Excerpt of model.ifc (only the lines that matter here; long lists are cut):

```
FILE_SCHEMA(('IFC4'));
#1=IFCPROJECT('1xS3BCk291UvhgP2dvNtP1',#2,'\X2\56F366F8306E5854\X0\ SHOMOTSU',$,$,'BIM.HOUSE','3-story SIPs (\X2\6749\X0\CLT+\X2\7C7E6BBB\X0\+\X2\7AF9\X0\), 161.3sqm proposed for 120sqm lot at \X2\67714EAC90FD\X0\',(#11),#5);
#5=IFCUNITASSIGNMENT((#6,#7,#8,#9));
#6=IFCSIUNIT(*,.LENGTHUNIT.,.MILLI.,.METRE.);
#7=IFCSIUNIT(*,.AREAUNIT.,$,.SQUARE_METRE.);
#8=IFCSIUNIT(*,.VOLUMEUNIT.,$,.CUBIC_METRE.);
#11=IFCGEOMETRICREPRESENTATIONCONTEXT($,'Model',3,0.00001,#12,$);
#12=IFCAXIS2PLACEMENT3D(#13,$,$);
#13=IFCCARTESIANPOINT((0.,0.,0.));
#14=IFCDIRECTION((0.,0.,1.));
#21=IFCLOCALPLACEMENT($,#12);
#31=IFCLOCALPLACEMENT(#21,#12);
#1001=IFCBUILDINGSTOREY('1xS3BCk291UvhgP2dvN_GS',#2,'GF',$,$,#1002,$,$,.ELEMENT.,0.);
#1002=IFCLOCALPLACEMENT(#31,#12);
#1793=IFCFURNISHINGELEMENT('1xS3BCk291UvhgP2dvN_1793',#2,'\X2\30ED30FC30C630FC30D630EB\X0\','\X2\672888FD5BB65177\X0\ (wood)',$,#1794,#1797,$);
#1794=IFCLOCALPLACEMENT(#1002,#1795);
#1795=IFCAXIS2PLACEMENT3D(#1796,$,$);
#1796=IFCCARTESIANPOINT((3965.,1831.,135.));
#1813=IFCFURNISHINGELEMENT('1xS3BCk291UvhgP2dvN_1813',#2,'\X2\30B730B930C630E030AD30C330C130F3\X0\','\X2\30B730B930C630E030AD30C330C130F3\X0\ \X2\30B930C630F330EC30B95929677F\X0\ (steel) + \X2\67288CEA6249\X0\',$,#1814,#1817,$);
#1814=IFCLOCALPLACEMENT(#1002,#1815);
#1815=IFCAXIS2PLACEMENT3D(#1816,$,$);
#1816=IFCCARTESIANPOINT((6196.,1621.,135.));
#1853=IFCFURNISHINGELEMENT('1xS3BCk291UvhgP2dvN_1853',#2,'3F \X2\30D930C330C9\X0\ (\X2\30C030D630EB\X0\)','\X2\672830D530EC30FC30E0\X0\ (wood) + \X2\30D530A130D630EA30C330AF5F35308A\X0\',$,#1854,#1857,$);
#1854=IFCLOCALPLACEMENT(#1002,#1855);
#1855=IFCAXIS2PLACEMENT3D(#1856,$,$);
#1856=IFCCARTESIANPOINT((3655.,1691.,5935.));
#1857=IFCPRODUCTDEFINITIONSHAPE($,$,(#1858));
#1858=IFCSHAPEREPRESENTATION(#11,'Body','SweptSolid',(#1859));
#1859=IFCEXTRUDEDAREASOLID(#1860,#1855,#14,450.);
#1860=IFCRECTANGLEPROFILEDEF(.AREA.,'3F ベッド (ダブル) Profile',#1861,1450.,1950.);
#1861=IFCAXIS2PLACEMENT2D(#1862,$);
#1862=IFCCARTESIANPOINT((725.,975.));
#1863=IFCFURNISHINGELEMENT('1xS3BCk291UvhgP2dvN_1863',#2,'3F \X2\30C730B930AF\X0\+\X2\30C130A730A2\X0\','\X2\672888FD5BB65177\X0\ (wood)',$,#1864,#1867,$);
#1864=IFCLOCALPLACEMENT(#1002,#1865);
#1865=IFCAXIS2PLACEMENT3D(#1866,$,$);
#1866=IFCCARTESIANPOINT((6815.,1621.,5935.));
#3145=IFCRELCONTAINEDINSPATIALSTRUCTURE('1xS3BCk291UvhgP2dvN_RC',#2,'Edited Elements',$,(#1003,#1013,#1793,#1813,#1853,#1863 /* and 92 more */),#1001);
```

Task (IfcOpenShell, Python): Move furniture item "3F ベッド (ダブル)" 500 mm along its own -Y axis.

```python
import ifcopenshell
import ifcopenshell.api.geometry
import ifcopenshell.util.placement
import ifcopenshell.util.unit

model = ifcopenshell.open("model.ifc")
unit_scale = ifcopenshell.util.unit.calculate_unit_scale(model)

item = model.by_guid("1xS3BCk291UvhgP2dvN_1853")
matrix = ifcopenshell.util.placement.get_local_placement(item.ObjectPlacement)
matrix[:3, 3] -= matrix[:3, 1] * 0.5 / unit_scale
ifcopenshell.api.geometry.edit_object_placement(model, product=item, matrix=matrix, is_si=False)

print(ifcopenshell.util.placement.get_local_placement(item.ObjectPlacement).round(3) + 0.0)

model.write("model_v2.ifc")
```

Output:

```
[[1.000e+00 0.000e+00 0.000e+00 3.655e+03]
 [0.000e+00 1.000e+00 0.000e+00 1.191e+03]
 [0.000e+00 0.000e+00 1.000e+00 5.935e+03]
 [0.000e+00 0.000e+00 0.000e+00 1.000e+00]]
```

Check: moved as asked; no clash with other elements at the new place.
